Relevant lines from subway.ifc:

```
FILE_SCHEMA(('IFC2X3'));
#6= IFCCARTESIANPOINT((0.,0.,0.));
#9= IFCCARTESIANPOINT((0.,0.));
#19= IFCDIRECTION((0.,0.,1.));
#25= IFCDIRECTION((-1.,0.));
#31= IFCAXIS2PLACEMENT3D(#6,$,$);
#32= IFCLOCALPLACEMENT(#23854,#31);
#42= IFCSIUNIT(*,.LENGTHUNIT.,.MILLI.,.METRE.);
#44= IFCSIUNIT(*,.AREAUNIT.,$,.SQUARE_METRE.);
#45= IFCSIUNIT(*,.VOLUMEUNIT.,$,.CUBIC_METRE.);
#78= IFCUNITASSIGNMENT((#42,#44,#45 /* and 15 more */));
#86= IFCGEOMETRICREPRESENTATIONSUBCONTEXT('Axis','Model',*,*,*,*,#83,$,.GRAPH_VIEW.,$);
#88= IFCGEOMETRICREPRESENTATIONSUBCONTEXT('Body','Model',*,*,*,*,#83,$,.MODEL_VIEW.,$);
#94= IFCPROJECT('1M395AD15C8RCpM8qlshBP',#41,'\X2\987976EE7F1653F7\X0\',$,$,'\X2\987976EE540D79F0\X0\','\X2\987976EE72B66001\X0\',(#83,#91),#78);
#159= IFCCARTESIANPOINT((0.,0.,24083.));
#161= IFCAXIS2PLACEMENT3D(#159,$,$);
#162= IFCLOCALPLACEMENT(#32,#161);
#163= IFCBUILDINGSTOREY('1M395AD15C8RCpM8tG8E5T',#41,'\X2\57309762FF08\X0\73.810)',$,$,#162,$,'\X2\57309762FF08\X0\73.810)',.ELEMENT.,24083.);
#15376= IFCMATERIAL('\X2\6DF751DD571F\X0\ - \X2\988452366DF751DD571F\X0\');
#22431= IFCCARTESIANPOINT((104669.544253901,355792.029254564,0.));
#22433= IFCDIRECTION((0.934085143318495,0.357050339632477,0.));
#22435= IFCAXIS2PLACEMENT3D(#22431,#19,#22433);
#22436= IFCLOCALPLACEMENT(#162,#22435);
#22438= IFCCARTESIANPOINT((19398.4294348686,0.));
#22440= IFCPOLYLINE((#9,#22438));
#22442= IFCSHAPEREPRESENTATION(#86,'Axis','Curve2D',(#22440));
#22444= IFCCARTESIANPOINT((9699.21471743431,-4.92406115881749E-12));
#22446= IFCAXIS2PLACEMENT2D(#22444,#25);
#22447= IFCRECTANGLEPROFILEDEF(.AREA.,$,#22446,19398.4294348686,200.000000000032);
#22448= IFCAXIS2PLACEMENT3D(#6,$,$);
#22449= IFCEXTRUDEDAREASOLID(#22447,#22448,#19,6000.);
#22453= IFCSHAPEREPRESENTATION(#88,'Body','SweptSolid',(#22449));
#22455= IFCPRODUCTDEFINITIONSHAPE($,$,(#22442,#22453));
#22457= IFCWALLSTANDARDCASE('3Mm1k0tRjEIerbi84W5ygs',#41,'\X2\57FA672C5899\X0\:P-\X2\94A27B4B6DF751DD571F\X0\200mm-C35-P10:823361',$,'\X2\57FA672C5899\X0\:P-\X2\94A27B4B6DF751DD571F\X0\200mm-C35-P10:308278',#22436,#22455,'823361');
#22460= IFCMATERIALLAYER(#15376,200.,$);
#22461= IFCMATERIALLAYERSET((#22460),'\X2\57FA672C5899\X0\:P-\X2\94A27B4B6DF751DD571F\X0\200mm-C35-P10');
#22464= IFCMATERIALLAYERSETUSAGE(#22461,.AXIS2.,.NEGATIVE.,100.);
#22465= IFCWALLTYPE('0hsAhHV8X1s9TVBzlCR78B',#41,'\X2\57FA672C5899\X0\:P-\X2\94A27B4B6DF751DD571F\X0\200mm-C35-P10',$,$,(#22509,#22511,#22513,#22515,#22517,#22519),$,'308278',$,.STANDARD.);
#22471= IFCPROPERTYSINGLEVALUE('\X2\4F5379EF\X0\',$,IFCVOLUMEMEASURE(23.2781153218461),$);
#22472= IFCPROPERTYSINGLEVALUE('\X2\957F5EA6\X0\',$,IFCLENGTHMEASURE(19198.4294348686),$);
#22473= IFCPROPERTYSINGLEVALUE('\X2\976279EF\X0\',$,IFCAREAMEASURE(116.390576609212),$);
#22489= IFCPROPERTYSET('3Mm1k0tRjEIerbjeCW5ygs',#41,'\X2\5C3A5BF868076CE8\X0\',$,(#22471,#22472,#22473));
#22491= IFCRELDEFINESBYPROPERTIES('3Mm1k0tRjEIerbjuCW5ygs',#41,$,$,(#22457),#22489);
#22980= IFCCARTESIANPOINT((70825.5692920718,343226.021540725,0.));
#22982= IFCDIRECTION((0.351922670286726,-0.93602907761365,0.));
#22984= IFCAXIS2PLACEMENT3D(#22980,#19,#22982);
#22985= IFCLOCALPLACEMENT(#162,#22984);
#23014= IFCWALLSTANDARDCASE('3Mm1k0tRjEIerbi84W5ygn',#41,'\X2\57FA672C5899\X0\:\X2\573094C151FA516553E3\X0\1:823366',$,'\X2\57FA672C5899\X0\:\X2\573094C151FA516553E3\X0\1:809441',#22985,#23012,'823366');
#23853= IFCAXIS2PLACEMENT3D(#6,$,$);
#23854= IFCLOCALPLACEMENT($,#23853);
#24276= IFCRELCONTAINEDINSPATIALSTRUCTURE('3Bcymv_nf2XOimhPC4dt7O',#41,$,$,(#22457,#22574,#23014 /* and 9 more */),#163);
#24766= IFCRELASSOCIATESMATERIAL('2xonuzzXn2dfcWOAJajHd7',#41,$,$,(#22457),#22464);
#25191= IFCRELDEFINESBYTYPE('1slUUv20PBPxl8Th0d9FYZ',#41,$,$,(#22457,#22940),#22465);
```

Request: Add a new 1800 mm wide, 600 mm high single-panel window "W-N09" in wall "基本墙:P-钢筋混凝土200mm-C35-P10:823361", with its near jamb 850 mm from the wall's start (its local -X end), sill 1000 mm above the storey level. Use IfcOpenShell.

```python
import numpy as np
import ifcopenshell
import ifcopenshell.api.feature
import ifcopenshell.api.geometry
import ifcopenshell.api.pset
import ifcopenshell.api.root
import ifcopenshell.api.spatial
import ifcopenshell.api.type
import ifcopenshell.geom
import ifcopenshell.util.element
import ifcopenshell.util.placement
import ifcopenshell.util.representation
import ifcopenshell.util.shape
import ifcopenshell.util.unit

model = ifcopenshell.open("subway.ifc")
unit_scale = ifcopenshell.util.unit.calculate_unit_scale(model)
area_scale = ifcopenshell.util.unit.calculate_unit_scale(model, "AREAUNIT")
volume_scale = ifcopenshell.util.unit.calculate_unit_scale(model, "VOLUMEUNIT")
settings = ifcopenshell.geom.settings()


def volume(element):
    """Net volume in cubic metres, openings subtracted."""
    shape = ifcopenshell.geom.create_shape(settings, element)
    return ifcopenshell.util.shape.get_volume(shape.geometry)


wall = model.by_guid("3Mm1k0tRjEIerbi84W5ygs")
storey = ifcopenshell.util.element.get_container(wall, ifc_class="IfcBuildingStorey")
context = ifcopenshell.util.representation.get_context(model, "Model", "Body", "MODEL_VIEW")
before = volume(wall)

width, height, from_end, sill = 1.8, 0.6, 0.85, 1  # metres

# The wall runs along its own X axis, and the end named is its -X end.
wall_shape = ifcopenshell.geom.create_shape(settings, wall)
x, y, z = ifcopenshell.util.shape.get_vertices(wall_shape.geometry).T
start = x.min() + from_end
face, thickness = float(y.min()), float(y.max() - y.min())
wall_matrix = ifcopenshell.util.placement.get_local_placement(wall.ObjectPlacement)
level = ifcopenshell.util.placement.get_local_placement(storey.ObjectPlacement)[2, 3]


def in_wall(x, y):
    """Placement at x, y metres in the wall's axes, at sill height."""
    matrix = wall_matrix.copy()
    matrix[:, 3] = wall_matrix @ np.array([x / unit_scale, y / unit_scale, 0.0, 1.0])
    matrix[2, 3] = level + sill / unit_scale
    return matrix


# Opening: a box that overshoots both wall faces by 50 mm.
opening = ifcopenshell.api.root.create_entity(model, ifc_class="IfcOpeningElement")
box = ifcopenshell.api.geometry.add_wall_representation(
    model, context=context, length=width, height=height, thickness=thickness + 0.1
)
ifcopenshell.api.geometry.assign_representation(model, product=opening, representation=box)
ifcopenshell.api.geometry.edit_object_placement(model, product=opening, matrix=in_wall(start, face - 0.05), is_si=False)
ifcopenshell.api.feature.add_feature(model, feature=opening, element=wall)

window = ifcopenshell.api.root.create_entity(model, ifc_class="IfcWindow", name="W-N09")
window.OverallWidth, window.OverallHeight = width / unit_scale, height / unit_scale
body = ifcopenshell.api.geometry.add_window_representation(
    model,
    context=context,
    overall_width=window.OverallWidth,
    overall_height=window.OverallHeight,
    partition_type="SINGLE_PANEL",
)
ifcopenshell.api.geometry.assign_representation(model, product=window, representation=body)
ifcopenshell.api.spatial.assign_container(model, products=[window], relating_structure=storey)
fills = ifcopenshell.api.feature.add_filling(model, opening=opening, element=window)
fills.OwnerHistory = window.OwnerHistory  # required in IFC2X3

# IFC2X3 keeps the operation on the window style.
style = ifcopenshell.api.root.create_entity(model, ifc_class="IfcWindowStyle", name="W-N09")
style.OperationType, style.ConstructionType = "SINGLE_PANEL", "NOTDEFINED"
style.ParameterTakesPrecedence = style.Sizeable = False
ifcopenshell.api.type.assign_type(model, related_objects=[window], relating_type=style)

# Centre the window in the wall's thickness.
ifcopenshell.api.geometry.edit_object_placement(model, product=window, matrix=in_wall(start, face), is_si=False)
window_shape = ifcopenshell.geom.create_shape(settings, window)
depth = ifcopenshell.util.shape.get_vertices(window_shape.geometry)[:, 1]
offset = face + thickness / 2 - (depth.min() + depth.max()) / 2
ifcopenshell.api.geometry.edit_object_placement(model, product=window, matrix=in_wall(start, offset), is_si=False)

after = volume(wall)

# Update the wall's stored quantities.
pset = model.by_id(ifcopenshell.util.element.get_pset(wall, "尺寸标注", should_inherit=False)["id"])
ifcopenshell.api.pset.edit_pset(model, pset=pset, properties={
    "体积": model.create_entity("IfcVolumeMeasure", after / volume_scale),
    "面积": model.create_entity("IfcAreaMeasure", after / thickness / area_scale),
})

print(f"wall volume {before:.3f} -> {after:.3f} m3")

model.write("subway_v2.ifc")
```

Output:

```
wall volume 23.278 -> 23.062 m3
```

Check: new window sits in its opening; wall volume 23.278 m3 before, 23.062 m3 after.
